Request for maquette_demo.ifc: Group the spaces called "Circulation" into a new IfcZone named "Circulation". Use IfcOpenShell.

First a look at what the model holds.

```python
import ifcopenshell

model = ifcopenshell.open("maquette_demo.ifc")
print(model.schema)
seen = {}
for space in model.by_type("IfcSpace"):
    seen[space.LongName] = seen.get(space.LongName, 0) + 1
for name, count in sorted(seen.items(), key=str):
    print(count, "x", name)
print("zones:", [z.Name for z in model.by_type("IfcZone")][:20])
```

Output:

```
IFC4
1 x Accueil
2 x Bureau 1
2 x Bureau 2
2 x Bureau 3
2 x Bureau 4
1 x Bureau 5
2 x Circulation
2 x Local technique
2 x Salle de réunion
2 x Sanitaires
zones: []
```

```python
import ifcopenshell
import ifcopenshell.api.group
import ifcopenshell.api.root

model = ifcopenshell.open("maquette_demo.ifc")

names = {"Circulation"}
spaces = [s for s in model.by_type("IfcSpace") if s.LongName in names]

zone = ifcopenshell.api.root.create_entity(model, ifc_class="IfcZone", name="Circulation")
ifcopenshell.api.group.assign_group(model, products=spaces, group=zone)
print(len(spaces), "spaces in", zone.Name)

model.write("maquette_demo_v2.ifc")
```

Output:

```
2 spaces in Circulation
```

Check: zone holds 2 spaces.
